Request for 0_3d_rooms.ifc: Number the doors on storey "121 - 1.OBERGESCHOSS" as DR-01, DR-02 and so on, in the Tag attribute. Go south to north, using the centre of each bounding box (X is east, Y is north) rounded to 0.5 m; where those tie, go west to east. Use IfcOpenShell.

First a look at what the model holds.

```python
import ifcopenshell
import ifcopenshell.util.element
import ifcopenshell.util.placement

model = ifcopenshell.open("0_3d_rooms.ifc")
print(model.schema)
storey = next(s for s in model.by_type("IfcBuildingStorey") if s.Name == "121 - 1.OBERGESCHOSS")
doors = [e for e in ifcopenshell.util.element.get_decomposition(storey) if e.is_a("IfcDoor")]
for e in sorted(doors, key=lambda e: e.id()):
    origin = ifcopenshell.util.placement.get_local_placement(e.ObjectPlacement)[:3, 3]
    print(e.id(), e.Tag, e.Name, origin.round(2) + 0.0, sep=" | ")
```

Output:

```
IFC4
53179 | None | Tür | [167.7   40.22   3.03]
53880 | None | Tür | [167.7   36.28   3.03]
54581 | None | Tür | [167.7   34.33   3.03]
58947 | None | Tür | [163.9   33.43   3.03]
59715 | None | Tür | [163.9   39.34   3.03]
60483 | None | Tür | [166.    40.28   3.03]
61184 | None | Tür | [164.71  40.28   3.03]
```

```python
import ifcopenshell
import ifcopenshell.geom
import ifcopenshell.util.element
import ifcopenshell.util.shape

model = ifcopenshell.open("0_3d_rooms.ifc")
settings = ifcopenshell.geom.settings()
settings.set("use-world-coords", True)


def centre(element):
    shape = ifcopenshell.geom.create_shape(settings, element)
    return ifcopenshell.util.shape.get_bbox_centroid(shape.geometry)


storey = next(s for s in model.by_type("IfcBuildingStorey") if s.Name == "121 - 1.OBERGESCHOSS")
doors = [e for e in ifcopenshell.util.element.get_decomposition(storey) if e.is_a("IfcDoor")]

# Insertion points can sit at a corner or the storey origin, so sort by the geometry (in metres).
centres = {e: centre(e) for e in doors}
doors.sort(key=lambda e: (round(centres[e][1] / 0.5), centres[e][0]))

for i, e in enumerate(doors, start=1):
    number = f"DR-{i:02d}"
    e.Tag = number
    print(e.id(), number)

model.write("0_3d_rooms_rev.ifc")
```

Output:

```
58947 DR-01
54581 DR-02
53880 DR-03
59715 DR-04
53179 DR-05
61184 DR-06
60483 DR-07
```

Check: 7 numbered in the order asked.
